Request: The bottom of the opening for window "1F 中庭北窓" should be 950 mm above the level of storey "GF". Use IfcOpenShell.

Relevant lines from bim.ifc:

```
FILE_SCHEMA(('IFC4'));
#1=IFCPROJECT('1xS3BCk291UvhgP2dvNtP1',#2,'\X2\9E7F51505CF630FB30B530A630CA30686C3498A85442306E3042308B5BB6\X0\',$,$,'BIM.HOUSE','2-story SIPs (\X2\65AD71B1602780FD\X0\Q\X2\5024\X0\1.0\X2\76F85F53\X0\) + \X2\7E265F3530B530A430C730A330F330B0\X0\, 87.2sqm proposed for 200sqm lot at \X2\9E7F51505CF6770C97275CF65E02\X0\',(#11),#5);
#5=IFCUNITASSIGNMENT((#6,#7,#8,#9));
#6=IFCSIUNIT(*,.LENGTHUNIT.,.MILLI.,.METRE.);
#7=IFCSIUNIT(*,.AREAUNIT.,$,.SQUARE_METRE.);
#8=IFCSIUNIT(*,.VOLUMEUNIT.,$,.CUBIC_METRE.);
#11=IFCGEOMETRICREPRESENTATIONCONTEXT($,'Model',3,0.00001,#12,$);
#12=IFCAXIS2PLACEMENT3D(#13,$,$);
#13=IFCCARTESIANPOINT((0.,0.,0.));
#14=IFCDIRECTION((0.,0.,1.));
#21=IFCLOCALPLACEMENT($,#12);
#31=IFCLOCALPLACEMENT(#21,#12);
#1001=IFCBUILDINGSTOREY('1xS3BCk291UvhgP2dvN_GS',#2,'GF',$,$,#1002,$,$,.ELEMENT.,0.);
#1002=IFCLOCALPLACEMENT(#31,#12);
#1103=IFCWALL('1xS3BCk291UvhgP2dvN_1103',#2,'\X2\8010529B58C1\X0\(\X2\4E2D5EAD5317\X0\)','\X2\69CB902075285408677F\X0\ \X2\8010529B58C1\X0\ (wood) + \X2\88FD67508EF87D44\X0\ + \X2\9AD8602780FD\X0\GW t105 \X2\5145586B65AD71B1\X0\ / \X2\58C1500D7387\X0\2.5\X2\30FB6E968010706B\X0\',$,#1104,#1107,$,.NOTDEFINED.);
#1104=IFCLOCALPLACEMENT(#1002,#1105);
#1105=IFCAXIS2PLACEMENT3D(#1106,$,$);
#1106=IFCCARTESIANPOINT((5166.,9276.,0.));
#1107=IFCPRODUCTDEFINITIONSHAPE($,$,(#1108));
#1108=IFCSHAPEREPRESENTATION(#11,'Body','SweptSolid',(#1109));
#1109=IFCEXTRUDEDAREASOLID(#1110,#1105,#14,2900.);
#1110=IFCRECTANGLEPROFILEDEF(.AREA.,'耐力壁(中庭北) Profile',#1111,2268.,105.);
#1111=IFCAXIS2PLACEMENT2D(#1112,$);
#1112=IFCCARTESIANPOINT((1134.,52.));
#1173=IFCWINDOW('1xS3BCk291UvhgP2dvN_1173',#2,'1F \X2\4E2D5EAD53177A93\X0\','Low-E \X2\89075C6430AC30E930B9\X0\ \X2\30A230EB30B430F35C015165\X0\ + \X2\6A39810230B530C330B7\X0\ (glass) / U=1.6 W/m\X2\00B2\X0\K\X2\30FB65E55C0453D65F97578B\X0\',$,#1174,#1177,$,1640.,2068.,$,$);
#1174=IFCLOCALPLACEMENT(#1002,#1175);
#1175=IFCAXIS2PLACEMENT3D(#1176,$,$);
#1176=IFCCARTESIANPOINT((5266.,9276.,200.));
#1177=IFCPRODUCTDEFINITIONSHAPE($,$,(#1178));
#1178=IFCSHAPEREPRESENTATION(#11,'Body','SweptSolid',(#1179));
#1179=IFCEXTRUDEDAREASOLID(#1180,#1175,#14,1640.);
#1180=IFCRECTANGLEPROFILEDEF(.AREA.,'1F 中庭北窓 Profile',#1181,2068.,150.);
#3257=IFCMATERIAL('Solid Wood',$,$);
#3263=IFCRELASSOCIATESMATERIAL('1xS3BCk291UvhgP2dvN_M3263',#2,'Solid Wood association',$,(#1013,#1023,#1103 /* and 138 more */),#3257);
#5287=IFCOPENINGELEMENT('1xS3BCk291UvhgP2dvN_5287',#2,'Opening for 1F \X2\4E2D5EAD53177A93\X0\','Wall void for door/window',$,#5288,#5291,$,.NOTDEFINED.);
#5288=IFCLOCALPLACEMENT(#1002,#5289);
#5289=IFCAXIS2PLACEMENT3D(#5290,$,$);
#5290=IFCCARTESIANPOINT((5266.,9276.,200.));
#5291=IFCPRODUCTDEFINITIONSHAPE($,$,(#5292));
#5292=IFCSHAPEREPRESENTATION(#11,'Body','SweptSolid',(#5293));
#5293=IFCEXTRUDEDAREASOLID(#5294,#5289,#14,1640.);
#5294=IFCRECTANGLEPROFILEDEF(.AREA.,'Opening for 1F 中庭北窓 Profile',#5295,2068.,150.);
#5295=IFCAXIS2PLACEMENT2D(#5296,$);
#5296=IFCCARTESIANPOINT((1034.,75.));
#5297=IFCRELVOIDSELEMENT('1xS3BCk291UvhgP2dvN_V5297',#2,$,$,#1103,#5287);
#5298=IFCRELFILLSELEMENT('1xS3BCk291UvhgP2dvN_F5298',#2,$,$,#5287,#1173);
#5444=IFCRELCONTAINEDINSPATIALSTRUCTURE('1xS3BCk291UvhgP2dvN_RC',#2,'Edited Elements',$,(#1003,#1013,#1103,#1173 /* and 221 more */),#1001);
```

```python
import numpy as np
import ifcopenshell
import ifcopenshell.api.geometry
import ifcopenshell.geom
import ifcopenshell.util.element
import ifcopenshell.util.placement
import ifcopenshell.util.shape
import ifcopenshell.util.unit

model = ifcopenshell.open("bim.ifc")
unit_scale = ifcopenshell.util.unit.calculate_unit_scale(model)

window = model.by_guid("1xS3BCk291UvhgP2dvN_1173")
opening = window.FillsVoids[0].RelatingOpeningElement
storey = ifcopenshell.util.element.get_container(window, ifc_class="IfcBuildingStorey")
level = ifcopenshell.util.placement.get_local_placement(storey.ObjectPlacement)[2, 3]

# The opening's origin need not be at the sill, so measure its lowest point.
shape = ifcopenshell.geom.create_shape(ifcopenshell.geom.settings(), opening)
bottom = ifcopenshell.util.shape.get_shape_bottom_elevation(shape, shape.geometry) / unit_scale
dz = level + 0.95 / unit_scale - bottom

shift = np.array([0.0, 0.0, dz])
# The window is not placed relative to its opening, so move both.
for product in (opening, window):
    matrix = ifcopenshell.util.placement.get_local_placement(product.ObjectPlacement)
    matrix[:3, 3] += shift
    ifcopenshell.api.geometry.edit_object_placement(model, product=product, matrix=matrix, is_si=False)

print(f"moved by {dz * unit_scale:+.3f} m")

model.write("bim_edited.ifc")
```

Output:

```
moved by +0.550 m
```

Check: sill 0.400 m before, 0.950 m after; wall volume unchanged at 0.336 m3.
